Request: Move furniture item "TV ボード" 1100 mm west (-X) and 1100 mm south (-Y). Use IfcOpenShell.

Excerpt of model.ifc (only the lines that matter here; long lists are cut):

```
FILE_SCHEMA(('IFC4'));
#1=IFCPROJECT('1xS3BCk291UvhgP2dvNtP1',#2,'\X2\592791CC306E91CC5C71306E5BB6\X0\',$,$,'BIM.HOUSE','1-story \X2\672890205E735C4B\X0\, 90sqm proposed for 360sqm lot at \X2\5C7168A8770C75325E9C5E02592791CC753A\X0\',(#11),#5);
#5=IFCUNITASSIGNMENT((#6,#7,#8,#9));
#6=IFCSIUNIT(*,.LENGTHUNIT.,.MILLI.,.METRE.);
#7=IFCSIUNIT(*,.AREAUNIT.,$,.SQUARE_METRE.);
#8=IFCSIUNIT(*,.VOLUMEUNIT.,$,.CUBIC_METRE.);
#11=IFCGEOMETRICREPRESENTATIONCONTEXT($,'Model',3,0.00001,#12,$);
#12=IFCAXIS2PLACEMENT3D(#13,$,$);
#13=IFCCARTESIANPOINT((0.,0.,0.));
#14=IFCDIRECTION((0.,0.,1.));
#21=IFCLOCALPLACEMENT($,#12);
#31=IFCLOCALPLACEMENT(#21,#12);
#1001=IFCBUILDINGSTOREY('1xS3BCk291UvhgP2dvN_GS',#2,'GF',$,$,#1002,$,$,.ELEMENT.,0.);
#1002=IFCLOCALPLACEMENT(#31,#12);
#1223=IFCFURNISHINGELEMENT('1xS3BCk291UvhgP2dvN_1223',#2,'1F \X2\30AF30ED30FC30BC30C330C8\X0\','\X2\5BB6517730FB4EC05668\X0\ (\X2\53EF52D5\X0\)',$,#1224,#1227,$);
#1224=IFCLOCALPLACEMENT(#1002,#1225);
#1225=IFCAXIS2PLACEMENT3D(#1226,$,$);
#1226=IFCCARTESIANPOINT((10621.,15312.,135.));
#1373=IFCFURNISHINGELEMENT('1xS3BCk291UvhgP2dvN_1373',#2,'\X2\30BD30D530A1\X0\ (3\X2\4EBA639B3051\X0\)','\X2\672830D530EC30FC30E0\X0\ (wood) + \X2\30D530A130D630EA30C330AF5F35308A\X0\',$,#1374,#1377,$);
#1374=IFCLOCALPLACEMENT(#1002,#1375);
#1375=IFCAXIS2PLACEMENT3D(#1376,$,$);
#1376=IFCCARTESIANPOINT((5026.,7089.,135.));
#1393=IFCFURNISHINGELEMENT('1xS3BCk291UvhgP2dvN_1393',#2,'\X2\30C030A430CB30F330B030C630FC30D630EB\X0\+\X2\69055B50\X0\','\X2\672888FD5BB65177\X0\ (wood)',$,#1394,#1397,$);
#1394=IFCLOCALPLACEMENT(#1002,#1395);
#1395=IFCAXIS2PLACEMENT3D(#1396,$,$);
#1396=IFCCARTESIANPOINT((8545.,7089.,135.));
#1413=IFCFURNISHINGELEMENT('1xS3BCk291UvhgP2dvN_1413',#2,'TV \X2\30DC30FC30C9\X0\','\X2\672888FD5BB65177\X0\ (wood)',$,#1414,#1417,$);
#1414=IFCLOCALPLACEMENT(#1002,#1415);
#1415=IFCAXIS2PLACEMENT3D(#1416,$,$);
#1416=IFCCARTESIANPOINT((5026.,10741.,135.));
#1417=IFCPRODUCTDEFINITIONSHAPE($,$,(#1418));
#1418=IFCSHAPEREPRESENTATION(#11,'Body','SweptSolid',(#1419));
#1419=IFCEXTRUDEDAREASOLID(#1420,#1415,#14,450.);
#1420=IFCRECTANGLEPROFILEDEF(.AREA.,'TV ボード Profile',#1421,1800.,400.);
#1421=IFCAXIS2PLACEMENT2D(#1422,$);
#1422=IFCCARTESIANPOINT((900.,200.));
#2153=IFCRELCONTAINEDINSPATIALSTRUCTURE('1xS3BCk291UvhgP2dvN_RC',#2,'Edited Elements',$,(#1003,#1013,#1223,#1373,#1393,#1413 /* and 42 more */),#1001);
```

```python
import ifcopenshell
import ifcopenshell.api.geometry
import ifcopenshell.util.placement

model = ifcopenshell.open("model.ifc")

item = model.by_guid("1xS3BCk291UvhgP2dvN_1413")
matrix = ifcopenshell.util.placement.get_local_placement(item.ObjectPlacement)
matrix[0, 3] -= 1100.0
matrix[1, 3] -= 1100.0
ifcopenshell.api.geometry.edit_object_placement(model, product=item, matrix=matrix, is_si=False)

print(ifcopenshell.util.placement.get_local_placement(item.ObjectPlacement).round(3) + 0.0)

model.write("model_v2.ifc")
```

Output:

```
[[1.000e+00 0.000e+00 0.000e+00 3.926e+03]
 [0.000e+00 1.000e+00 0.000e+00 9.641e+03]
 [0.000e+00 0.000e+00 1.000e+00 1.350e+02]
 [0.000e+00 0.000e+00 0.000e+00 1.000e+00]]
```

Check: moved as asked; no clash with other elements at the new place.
